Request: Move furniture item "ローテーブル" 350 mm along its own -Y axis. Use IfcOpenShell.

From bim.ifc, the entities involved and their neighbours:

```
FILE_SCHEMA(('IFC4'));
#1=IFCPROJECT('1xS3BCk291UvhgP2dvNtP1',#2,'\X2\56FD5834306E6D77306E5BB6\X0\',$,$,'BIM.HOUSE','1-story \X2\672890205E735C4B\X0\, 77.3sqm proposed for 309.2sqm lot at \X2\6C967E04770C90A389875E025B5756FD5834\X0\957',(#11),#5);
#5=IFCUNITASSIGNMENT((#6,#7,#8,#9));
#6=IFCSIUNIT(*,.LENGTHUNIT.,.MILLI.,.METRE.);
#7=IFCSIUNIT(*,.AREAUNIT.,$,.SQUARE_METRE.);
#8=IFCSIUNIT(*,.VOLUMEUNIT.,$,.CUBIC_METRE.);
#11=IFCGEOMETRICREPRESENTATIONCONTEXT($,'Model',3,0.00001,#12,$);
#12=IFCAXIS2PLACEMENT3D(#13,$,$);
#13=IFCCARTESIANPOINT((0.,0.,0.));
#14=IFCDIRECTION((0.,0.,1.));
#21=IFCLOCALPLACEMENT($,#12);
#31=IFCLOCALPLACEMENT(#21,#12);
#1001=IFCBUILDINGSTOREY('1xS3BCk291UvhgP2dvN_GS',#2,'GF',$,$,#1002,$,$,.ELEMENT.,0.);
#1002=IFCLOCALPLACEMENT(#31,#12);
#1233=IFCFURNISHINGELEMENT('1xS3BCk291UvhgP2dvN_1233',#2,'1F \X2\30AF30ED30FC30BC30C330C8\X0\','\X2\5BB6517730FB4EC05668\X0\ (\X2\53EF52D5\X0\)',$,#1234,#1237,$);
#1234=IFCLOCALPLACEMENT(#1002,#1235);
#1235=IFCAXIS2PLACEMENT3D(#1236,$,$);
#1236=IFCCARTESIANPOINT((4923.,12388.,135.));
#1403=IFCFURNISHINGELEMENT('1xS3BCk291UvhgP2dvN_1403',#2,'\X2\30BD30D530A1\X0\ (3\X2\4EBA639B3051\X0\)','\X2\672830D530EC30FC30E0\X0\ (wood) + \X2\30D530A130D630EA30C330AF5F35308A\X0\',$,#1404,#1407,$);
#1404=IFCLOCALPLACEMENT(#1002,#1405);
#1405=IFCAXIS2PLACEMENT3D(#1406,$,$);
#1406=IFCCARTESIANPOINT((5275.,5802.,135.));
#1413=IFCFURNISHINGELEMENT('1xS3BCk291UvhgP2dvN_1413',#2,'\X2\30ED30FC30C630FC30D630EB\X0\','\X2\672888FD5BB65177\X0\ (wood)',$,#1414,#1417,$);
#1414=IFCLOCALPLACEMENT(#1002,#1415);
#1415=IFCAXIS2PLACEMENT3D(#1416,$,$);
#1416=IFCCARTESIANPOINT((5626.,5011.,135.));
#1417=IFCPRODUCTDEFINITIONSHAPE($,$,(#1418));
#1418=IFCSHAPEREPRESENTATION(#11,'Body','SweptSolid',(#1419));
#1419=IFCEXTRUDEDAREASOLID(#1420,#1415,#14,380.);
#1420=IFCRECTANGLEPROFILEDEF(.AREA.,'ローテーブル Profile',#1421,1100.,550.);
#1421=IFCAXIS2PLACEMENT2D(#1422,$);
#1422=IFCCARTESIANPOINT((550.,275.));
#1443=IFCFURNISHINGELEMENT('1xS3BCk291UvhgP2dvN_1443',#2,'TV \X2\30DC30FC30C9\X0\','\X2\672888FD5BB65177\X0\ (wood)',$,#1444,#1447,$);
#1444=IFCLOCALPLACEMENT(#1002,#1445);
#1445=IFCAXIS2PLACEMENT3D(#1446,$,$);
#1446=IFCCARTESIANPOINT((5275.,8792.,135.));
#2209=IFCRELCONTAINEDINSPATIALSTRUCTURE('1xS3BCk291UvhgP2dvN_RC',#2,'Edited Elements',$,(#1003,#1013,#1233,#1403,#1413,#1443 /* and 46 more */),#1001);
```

```python
import ifcopenshell
import ifcopenshell.api.geometry
import ifcopenshell.util.placement
import ifcopenshell.util.unit

model = ifcopenshell.open("bim.ifc")
unit_scale = ifcopenshell.util.unit.calculate_unit_scale(model)

item = model.by_guid("1xS3BCk291UvhgP2dvN_1413")
matrix = ifcopenshell.util.placement.get_local_placement(item.ObjectPlacement)
matrix[:3, 3] -= matrix[:3, 1] * 0.35 / unit_scale
ifcopenshell.api.geometry.edit_object_placement(model, product=item, matrix=matrix, is_si=False)

print(ifcopenshell.util.placement.get_local_placement(item.ObjectPlacement).round(3) + 0.0)

model.write("bim-out.ifc")
```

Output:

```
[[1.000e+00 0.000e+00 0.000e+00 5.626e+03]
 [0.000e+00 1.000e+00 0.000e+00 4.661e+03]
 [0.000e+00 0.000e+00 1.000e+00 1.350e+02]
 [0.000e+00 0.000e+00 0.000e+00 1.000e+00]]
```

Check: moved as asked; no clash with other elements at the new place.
